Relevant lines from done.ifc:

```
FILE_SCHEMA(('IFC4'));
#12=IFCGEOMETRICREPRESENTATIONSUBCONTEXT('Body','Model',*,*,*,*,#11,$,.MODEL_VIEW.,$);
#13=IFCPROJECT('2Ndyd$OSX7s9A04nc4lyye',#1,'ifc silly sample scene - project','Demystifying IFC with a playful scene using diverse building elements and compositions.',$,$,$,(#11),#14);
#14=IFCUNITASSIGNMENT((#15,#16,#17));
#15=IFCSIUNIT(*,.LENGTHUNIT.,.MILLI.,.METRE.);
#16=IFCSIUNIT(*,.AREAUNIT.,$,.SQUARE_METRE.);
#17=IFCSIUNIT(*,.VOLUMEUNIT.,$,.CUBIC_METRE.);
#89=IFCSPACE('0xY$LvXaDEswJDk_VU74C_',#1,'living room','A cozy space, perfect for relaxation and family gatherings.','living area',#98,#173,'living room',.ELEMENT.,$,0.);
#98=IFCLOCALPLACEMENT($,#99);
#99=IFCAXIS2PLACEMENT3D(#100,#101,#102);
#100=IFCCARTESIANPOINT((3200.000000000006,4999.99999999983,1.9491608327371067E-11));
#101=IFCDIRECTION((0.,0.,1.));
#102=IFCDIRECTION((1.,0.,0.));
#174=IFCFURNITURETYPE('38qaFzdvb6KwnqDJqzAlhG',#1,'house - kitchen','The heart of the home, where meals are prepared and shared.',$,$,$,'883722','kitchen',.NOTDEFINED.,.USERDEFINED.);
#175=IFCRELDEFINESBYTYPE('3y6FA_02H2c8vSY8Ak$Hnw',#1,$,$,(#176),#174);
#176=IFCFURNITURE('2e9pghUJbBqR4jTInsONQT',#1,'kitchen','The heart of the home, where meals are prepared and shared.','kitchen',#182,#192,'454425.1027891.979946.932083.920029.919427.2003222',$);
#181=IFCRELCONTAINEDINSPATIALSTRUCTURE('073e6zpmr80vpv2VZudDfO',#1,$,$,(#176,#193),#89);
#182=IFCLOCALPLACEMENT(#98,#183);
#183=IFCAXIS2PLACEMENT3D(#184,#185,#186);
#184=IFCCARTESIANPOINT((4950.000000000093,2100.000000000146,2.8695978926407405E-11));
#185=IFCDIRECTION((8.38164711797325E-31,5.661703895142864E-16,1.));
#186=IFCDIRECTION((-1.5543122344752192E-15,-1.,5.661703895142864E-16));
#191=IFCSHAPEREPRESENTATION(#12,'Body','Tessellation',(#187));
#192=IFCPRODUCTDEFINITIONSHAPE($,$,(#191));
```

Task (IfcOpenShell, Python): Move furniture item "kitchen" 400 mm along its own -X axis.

```python
import ifcopenshell
import ifcopenshell.api.geometry
import ifcopenshell.util.placement

model = ifcopenshell.open("done.ifc")

item = model.by_guid("2e9pghUJbBqR4jTInsONQT")
matrix = ifcopenshell.util.placement.get_local_placement(item.ObjectPlacement)
matrix[:3, 3] -= matrix[:3, 0] * 400.0
ifcopenshell.api.geometry.edit_object_placement(model, product=item, matrix=matrix, is_si=False)

print(ifcopenshell.util.placement.get_local_placement(item.ObjectPlacement).round(3) + 0.0)

model.write("done_rev.ifc")
```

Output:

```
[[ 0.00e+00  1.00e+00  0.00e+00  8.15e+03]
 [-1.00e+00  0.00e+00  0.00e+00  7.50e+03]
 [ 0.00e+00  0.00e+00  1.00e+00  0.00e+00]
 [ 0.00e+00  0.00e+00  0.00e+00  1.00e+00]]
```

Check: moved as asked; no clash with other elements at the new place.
